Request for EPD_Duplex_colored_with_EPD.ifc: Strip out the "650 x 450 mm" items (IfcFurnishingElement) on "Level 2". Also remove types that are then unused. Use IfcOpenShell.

First a look at what the model holds.

```python
import ifcopenshell
import ifcopenshell.util.element

model = ifcopenshell.open("EPD_Duplex_colored_with_EPD.ifc")
print(model.schema)
storey = next(s for s in model.by_type("IfcBuildingStorey") if s.Name == "Level 2")
furniture = [e for e in ifcopenshell.util.element.get_decomposition(storey) if e.is_a("IfcFurnishingElement")]
seen = {}
for e in furniture:
    element_type = ifcopenshell.util.element.get_type(e)
    name = element_type.Name if element_type not in (None, e) else None
    seen[name] = seen.get(name, 0) + 1
for name, count in sorted(seen.items(), key=str):
    print(count, "x", name)
```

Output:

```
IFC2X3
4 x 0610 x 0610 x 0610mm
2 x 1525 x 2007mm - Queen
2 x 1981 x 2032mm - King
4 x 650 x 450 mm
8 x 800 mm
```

```python
import ifcopenshell
import ifcopenshell.api.root
import ifcopenshell.util.element

model = ifcopenshell.open("EPD_Duplex_colored_with_EPD.ifc")

storey = next(s for s in model.by_type("IfcBuildingStorey") if s.Name == "Level 2")
furniture = [e for e in ifcopenshell.util.element.get_decomposition(storey) if e.is_a("IfcFurnishingElement")]
targets = [e for e in furniture if (t := ifcopenshell.util.element.get_type(e)) not in (None, e) and t.Name == "650 x 450 mm"]
types = {ifcopenshell.util.element.get_type(e) for e in targets} - {None, *targets}

for e in targets:
    ifcopenshell.api.root.remove_product(model, product=e)
print(len(targets), "removed")

unused = [t for t in types if not ifcopenshell.util.element.get_types(t)]
for t in unused:
    ifcopenshell.api.root.remove_product(model, product=t)
print(len(unused), "unused types removed")

model.write("EPD_Duplex_colored_with_EPD-out.ifc")
```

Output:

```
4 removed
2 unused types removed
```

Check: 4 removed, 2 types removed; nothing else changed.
